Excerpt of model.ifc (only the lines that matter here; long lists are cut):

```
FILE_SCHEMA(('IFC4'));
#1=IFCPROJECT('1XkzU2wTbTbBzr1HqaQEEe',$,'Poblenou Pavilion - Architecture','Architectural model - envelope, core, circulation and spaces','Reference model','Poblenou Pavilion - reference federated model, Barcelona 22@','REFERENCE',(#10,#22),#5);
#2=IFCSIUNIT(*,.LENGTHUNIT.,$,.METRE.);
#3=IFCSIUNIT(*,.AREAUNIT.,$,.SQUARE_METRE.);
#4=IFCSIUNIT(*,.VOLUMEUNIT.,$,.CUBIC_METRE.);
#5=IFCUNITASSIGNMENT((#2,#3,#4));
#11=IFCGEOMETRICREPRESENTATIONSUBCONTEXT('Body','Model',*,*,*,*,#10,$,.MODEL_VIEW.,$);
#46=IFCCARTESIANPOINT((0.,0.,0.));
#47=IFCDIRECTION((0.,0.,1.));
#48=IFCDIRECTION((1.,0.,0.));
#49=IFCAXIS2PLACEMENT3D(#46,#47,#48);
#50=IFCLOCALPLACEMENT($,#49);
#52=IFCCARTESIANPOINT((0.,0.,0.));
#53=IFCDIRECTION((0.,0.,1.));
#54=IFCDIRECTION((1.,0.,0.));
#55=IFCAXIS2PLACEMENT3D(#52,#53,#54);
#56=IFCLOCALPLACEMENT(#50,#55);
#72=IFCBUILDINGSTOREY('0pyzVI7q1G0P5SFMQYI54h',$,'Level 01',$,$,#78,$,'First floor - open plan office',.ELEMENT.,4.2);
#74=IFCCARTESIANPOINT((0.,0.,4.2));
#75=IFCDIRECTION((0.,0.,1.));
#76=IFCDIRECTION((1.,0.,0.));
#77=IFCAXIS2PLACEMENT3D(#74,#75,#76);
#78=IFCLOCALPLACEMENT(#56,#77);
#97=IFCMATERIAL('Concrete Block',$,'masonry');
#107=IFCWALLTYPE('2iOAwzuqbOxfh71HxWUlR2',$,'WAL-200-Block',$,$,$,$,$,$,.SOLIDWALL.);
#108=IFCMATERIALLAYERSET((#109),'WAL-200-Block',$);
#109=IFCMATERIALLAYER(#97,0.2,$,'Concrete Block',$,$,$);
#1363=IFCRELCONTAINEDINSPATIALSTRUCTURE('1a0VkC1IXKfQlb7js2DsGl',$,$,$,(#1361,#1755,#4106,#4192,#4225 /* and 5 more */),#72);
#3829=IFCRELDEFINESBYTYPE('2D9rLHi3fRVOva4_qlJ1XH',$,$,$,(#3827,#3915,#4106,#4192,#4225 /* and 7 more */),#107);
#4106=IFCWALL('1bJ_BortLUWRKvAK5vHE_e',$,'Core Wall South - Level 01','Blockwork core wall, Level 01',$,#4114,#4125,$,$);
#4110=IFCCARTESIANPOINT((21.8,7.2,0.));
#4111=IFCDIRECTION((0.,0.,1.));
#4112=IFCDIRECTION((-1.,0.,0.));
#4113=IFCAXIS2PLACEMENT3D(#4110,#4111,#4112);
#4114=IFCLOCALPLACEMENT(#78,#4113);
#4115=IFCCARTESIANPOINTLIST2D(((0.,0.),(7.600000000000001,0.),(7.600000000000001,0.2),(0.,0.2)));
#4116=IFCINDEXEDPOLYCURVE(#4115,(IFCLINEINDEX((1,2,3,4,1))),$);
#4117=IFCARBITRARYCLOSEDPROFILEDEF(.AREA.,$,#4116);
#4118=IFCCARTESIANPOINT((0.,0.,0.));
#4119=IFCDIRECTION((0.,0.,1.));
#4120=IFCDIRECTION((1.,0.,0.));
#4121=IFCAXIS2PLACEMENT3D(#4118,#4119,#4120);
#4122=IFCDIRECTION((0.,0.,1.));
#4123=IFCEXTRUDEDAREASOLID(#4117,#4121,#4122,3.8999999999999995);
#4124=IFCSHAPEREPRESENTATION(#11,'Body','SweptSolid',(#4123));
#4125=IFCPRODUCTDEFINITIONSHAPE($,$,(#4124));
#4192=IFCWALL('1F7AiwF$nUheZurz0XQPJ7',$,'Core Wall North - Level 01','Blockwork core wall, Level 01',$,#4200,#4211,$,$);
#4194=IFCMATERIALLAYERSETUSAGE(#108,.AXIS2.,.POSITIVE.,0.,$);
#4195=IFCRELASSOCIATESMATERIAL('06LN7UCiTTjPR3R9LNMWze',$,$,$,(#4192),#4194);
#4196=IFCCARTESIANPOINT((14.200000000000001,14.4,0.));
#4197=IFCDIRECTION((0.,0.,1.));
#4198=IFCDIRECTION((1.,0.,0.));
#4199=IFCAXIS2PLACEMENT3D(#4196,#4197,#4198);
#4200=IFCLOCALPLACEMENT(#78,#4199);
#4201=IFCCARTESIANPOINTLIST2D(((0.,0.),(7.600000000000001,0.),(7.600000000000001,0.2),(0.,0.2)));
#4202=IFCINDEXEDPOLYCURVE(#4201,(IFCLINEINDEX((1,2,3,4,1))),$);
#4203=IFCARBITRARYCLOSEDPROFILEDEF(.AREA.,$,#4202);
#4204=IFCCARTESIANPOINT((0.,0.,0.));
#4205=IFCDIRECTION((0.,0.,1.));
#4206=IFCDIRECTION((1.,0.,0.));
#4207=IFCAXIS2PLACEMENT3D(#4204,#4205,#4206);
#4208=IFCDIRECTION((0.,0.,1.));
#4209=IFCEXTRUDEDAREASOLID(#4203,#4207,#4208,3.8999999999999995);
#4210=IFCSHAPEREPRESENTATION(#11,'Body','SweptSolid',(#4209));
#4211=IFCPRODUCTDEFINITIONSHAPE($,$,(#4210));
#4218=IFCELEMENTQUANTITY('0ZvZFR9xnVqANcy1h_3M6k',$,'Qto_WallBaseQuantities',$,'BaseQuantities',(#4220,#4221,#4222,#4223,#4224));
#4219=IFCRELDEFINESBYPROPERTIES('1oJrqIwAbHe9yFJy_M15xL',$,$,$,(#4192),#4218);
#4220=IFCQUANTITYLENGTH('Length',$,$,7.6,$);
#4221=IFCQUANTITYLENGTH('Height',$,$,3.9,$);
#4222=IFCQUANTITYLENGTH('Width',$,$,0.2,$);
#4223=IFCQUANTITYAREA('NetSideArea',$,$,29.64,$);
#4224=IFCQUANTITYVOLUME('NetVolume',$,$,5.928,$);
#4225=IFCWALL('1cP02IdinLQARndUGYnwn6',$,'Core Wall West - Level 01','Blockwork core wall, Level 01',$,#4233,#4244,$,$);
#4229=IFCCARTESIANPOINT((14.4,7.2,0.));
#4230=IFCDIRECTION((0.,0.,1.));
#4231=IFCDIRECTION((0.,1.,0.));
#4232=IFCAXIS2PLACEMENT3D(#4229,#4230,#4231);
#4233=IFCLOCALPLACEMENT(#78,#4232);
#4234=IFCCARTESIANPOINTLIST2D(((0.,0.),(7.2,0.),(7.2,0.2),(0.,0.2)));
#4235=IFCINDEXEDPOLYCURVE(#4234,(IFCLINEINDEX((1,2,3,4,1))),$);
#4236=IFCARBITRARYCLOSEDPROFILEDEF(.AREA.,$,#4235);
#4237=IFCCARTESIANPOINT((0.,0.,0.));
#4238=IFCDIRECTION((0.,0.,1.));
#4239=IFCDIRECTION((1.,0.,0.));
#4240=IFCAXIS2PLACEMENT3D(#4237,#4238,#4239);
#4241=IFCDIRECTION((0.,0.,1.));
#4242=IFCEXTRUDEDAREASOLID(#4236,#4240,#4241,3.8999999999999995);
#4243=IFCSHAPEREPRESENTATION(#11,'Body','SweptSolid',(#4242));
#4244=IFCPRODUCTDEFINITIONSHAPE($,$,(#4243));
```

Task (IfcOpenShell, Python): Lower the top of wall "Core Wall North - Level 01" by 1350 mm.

```python
import ifcopenshell
import ifcopenshell.api.pset
import ifcopenshell.geom
import ifcopenshell.util.element
import ifcopenshell.util.representation
import ifcopenshell.util.shape
import ifcopenshell.util.unit

model = ifcopenshell.open("model.ifc")
area_scale = ifcopenshell.util.unit.calculate_unit_scale(model, "AREAUNIT")
volume_scale = ifcopenshell.util.unit.calculate_unit_scale(model, "VOLUMEUNIT")
settings = ifcopenshell.geom.settings()


def volume(element):
    """Net volume in cubic metres, openings subtracted."""
    shape = ifcopenshell.geom.create_shape(settings, element)
    return ifcopenshell.util.shape.get_volume(shape.geometry)


wall = model.by_guid("1F7AiwF$nUheZurz0XQPJ7")
before = volume(wall)

body = ifcopenshell.util.representation.get_representation(wall, "Model", "Body")
solid = body.Items[0]
old_height = solid.Depth
solid.Depth -= 1.35
after = volume(wall)
thickness = 0.2  # wall thickness in metres

# Update the stored height, areas and volumes.
qto = model.by_id(ifcopenshell.util.element.get_pset(wall, "Qto_WallBaseQuantities", should_inherit=False)["id"])
ifcopenshell.api.pset.edit_qto(model, qto=qto, properties={
    "Height": solid.Depth,
    "NetSideArea": after / thickness / area_scale,
    "NetVolume": after / volume_scale,
})

print(f"height {old_height:g} -> {solid.Depth:g}, volume {before:.3f} -> {after:.3f} m3")

model.write("model_edited.ifc")
```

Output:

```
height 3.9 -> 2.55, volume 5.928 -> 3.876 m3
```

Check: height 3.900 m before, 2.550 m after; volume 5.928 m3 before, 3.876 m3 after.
